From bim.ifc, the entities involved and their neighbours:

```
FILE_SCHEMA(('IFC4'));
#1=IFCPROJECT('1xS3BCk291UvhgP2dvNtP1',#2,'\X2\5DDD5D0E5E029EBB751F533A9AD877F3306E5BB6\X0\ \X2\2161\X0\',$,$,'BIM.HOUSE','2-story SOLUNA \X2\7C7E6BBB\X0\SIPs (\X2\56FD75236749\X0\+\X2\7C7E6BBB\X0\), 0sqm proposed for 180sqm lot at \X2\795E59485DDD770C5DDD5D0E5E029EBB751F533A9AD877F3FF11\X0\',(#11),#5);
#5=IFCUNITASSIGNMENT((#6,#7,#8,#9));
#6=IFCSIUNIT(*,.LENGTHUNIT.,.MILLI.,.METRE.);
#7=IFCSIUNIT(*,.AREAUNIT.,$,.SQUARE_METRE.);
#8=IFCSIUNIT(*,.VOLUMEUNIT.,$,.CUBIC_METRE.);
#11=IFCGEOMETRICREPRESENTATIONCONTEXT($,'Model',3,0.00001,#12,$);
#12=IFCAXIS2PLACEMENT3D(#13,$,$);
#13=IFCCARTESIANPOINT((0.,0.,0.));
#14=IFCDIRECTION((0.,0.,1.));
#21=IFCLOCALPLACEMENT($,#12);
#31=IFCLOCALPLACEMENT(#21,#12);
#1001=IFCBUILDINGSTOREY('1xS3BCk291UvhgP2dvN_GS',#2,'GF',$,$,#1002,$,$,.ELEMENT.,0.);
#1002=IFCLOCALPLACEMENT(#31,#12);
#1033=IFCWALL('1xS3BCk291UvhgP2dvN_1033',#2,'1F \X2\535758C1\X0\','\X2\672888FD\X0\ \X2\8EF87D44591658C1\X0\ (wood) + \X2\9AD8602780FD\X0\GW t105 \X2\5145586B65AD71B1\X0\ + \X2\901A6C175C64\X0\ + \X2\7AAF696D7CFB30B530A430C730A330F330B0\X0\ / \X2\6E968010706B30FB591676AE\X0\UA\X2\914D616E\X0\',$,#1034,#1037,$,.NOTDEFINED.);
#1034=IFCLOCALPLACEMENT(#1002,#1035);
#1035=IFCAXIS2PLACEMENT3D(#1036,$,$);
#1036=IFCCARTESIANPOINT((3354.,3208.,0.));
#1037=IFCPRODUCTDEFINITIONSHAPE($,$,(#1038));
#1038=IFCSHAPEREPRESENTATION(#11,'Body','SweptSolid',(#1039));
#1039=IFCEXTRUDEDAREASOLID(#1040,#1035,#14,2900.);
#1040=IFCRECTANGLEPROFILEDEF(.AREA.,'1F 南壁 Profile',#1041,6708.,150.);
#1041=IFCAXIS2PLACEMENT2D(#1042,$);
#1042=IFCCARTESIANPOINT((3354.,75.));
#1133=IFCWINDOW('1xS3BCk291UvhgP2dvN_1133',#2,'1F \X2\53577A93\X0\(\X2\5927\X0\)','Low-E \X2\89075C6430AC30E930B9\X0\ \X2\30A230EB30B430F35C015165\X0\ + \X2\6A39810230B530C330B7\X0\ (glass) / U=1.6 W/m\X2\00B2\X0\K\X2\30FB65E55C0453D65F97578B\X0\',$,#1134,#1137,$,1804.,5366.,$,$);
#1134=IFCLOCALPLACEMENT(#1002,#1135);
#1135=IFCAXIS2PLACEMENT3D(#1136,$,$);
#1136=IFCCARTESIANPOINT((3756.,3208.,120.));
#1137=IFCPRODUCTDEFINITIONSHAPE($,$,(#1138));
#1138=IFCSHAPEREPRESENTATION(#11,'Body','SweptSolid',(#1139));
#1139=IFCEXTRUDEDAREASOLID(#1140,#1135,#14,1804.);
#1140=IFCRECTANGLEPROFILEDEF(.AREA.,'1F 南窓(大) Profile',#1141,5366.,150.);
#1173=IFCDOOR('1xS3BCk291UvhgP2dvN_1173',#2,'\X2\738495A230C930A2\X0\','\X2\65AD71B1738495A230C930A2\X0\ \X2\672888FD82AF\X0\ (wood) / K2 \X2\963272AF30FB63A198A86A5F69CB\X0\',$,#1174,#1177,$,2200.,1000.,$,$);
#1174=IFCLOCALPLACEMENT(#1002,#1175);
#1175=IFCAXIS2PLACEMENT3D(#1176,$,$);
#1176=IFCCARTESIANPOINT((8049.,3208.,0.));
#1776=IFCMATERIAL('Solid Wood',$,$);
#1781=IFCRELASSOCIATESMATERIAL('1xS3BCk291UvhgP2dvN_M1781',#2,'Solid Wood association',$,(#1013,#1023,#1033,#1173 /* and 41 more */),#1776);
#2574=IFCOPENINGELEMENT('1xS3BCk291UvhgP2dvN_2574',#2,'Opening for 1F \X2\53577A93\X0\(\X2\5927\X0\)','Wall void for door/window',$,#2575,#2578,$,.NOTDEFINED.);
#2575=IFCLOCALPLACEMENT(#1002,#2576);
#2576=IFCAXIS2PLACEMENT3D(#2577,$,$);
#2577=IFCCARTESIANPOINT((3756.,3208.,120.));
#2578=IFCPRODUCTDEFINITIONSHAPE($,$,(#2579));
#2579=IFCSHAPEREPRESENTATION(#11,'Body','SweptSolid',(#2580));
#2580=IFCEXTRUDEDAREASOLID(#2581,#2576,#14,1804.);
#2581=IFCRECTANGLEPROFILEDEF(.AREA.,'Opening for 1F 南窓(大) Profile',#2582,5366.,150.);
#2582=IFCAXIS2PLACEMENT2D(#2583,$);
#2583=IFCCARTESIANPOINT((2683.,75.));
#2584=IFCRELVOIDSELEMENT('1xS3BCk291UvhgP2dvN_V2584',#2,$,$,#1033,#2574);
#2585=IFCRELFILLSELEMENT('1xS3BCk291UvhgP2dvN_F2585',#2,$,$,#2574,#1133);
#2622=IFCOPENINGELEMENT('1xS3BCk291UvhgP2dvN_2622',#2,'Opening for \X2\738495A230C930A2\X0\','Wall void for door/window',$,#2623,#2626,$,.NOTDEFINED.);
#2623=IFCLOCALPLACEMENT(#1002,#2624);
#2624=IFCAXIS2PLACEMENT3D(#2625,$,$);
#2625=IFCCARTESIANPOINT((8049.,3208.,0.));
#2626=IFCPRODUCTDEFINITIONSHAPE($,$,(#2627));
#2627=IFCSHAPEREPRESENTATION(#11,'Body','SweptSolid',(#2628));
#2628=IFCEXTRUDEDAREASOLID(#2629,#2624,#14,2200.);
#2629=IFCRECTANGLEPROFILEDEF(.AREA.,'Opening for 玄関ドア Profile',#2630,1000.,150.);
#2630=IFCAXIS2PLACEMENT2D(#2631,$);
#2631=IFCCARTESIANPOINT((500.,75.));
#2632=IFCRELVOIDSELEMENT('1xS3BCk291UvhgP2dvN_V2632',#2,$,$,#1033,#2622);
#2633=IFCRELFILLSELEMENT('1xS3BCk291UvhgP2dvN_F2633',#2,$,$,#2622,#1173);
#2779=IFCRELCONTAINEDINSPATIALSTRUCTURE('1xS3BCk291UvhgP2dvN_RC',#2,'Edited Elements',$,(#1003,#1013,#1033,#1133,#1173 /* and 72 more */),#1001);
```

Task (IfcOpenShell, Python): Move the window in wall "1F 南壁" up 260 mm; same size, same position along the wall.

```python
import numpy as np
import ifcopenshell
import ifcopenshell.api.geometry
import ifcopenshell.util.placement
import ifcopenshell.util.unit

model = ifcopenshell.open("bim.ifc")
unit_scale = ifcopenshell.util.unit.calculate_unit_scale(model)

window = model.by_guid("1xS3BCk291UvhgP2dvN_1133")
opening = window.FillsVoids[0].RelatingOpeningElement
dz = 260.0

shift = np.array([0.0, 0.0, dz])
# The window is not placed relative to its opening, so move both.
for product in (opening, window):
    matrix = ifcopenshell.util.placement.get_local_placement(product.ObjectPlacement)
    matrix[:3, 3] += shift
    ifcopenshell.api.geometry.edit_object_placement(model, product=product, matrix=matrix, is_si=False)

print(f"moved by {dz * unit_scale:+.3f} m")

model.write("bim_updated.ifc")
```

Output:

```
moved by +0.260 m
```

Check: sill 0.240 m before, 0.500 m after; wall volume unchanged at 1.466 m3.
